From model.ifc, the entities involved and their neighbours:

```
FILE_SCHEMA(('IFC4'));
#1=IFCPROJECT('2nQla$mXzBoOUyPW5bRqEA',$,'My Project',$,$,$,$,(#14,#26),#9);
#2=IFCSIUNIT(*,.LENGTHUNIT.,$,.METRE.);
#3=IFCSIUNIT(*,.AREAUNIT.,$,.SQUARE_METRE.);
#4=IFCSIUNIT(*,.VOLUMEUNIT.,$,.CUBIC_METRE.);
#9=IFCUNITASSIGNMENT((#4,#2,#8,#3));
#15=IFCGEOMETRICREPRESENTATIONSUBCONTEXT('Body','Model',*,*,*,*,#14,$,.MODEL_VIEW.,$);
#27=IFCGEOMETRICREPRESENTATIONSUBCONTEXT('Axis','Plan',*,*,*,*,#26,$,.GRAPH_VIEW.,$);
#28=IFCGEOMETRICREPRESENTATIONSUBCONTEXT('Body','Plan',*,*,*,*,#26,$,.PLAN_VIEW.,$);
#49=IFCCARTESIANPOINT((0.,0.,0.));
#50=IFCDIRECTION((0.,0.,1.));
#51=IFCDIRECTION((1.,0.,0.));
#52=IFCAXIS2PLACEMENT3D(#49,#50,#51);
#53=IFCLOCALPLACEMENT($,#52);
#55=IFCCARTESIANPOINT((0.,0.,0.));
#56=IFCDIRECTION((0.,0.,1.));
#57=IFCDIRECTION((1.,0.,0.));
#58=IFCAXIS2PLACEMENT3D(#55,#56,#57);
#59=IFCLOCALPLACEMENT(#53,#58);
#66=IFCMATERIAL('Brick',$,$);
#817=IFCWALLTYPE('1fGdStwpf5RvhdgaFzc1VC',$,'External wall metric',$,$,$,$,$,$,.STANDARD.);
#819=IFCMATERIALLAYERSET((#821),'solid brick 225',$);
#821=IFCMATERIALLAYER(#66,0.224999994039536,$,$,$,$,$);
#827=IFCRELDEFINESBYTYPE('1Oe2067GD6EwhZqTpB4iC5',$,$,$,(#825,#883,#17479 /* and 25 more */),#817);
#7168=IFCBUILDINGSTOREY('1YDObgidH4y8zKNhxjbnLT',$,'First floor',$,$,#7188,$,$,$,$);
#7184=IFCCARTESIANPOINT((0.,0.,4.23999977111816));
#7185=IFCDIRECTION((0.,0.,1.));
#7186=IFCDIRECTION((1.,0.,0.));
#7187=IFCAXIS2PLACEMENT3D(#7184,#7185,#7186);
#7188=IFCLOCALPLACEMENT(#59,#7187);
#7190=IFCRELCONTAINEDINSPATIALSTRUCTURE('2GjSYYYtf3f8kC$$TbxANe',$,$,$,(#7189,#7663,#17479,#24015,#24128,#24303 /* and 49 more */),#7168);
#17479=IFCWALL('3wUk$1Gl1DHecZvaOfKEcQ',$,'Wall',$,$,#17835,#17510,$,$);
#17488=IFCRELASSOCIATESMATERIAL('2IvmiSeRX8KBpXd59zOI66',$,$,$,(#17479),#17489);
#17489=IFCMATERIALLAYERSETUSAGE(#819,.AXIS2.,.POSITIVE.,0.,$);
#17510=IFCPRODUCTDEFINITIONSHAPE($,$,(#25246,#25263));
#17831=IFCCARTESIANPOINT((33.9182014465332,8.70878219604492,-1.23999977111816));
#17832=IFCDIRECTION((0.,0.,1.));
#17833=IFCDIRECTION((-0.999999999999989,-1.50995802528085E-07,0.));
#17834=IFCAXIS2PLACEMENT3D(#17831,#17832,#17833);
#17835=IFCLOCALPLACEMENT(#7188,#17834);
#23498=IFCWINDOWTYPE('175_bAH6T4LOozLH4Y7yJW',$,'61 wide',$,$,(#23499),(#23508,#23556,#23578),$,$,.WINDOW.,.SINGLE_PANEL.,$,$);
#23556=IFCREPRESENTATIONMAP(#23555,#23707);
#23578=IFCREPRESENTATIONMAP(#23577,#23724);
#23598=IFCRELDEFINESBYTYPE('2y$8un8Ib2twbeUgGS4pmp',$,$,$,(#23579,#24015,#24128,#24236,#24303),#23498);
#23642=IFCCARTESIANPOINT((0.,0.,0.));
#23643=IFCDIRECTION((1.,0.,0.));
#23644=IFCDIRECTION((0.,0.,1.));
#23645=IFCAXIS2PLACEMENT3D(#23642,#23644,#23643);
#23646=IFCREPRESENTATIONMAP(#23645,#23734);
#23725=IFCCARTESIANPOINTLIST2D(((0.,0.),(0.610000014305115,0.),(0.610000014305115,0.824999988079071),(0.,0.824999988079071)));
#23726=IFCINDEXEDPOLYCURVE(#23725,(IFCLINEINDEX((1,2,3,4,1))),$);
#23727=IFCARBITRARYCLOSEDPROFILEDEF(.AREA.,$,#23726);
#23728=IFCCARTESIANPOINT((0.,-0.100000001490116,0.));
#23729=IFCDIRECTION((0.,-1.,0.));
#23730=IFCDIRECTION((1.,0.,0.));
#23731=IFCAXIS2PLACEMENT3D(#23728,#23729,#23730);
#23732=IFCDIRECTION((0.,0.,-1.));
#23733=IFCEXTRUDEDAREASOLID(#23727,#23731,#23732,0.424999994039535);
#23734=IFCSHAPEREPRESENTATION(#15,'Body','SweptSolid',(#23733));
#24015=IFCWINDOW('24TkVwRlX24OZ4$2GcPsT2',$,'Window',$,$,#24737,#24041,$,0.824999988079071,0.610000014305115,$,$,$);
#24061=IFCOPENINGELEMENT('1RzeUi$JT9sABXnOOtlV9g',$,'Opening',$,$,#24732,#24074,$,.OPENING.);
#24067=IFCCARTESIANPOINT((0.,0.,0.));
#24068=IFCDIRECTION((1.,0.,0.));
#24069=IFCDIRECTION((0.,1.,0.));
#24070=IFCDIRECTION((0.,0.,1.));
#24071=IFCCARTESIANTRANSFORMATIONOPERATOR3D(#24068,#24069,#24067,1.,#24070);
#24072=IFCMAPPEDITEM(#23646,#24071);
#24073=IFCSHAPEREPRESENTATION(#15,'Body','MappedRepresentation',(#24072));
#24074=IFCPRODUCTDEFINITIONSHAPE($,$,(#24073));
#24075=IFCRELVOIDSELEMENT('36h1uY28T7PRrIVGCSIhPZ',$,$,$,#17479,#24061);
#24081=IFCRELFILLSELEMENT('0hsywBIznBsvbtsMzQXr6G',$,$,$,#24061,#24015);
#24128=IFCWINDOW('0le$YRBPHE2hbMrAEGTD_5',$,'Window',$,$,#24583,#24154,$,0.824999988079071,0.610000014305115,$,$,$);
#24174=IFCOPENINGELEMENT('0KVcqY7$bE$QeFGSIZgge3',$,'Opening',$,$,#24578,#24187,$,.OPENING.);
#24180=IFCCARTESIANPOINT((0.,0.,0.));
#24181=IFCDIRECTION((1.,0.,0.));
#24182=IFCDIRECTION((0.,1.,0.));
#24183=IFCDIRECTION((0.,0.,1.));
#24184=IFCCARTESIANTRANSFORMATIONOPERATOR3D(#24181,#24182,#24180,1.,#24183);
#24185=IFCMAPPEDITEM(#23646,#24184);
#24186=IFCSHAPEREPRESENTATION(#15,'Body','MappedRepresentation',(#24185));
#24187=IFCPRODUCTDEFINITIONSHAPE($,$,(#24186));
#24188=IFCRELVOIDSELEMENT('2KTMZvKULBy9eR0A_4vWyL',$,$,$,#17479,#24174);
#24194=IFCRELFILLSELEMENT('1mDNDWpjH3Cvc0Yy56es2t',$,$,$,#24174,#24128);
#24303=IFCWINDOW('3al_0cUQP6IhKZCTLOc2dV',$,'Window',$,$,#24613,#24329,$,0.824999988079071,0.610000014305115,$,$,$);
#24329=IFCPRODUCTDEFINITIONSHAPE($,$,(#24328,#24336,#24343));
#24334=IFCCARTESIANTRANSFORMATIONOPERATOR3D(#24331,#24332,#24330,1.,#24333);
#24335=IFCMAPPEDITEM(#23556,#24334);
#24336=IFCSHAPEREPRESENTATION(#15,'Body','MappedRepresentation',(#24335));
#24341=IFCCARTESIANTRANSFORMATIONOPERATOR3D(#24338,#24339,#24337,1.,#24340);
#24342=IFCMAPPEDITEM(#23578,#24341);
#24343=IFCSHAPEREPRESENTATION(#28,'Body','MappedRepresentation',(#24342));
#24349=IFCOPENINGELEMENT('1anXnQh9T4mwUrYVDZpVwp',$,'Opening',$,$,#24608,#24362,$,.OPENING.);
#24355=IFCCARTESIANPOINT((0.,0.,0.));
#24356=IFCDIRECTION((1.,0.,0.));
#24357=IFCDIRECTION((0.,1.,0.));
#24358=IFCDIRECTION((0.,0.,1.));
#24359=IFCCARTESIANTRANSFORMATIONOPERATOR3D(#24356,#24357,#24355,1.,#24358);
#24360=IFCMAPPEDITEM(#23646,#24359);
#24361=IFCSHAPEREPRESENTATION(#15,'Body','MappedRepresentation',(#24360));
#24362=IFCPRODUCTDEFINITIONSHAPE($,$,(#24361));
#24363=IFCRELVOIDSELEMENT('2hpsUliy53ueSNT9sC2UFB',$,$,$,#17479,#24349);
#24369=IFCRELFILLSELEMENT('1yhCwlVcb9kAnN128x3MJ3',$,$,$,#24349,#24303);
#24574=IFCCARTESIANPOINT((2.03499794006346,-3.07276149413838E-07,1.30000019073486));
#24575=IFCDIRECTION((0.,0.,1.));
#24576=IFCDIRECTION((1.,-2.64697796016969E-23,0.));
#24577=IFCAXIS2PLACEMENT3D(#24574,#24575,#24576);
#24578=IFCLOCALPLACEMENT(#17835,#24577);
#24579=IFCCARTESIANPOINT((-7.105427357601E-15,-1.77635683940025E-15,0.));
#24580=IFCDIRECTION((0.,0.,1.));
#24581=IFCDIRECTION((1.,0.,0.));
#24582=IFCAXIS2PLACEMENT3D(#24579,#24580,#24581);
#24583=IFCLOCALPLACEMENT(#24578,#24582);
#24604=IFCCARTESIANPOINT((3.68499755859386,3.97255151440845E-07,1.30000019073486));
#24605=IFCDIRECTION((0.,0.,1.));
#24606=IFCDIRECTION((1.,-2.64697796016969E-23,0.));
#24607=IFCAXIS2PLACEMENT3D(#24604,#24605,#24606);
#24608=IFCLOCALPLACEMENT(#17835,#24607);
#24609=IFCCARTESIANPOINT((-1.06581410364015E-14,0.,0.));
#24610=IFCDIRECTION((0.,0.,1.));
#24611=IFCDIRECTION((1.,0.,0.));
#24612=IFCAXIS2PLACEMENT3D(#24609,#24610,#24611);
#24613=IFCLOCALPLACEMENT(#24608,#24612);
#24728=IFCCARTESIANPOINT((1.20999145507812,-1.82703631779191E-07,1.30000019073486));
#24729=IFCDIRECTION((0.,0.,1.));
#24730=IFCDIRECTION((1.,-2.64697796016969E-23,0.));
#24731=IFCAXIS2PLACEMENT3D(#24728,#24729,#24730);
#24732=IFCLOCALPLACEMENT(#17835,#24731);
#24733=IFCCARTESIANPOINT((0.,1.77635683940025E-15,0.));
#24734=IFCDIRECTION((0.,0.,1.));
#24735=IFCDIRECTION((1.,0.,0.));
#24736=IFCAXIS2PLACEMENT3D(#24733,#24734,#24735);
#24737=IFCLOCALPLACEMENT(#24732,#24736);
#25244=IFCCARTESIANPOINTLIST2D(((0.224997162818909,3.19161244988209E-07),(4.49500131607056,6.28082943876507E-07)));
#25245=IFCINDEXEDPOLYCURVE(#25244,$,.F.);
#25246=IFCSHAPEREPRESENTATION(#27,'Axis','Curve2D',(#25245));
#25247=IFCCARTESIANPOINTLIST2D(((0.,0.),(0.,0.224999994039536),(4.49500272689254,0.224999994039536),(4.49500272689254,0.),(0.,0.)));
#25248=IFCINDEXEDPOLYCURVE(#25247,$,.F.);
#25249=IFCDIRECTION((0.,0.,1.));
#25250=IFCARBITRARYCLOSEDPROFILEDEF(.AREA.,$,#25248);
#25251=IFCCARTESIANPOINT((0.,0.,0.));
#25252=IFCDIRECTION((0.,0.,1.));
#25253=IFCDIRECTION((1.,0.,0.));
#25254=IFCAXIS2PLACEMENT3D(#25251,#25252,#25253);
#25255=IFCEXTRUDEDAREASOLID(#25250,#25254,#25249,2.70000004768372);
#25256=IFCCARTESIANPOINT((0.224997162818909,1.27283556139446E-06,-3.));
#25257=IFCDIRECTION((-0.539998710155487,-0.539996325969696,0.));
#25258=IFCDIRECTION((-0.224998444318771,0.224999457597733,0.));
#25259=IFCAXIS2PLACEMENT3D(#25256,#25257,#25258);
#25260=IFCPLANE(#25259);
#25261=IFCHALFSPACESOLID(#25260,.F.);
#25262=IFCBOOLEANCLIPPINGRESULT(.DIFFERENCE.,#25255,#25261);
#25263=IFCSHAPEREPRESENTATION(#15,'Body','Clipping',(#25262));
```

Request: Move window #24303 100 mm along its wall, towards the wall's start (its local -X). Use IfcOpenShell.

```python
import ifcopenshell
import ifcopenshell.api.geometry
import ifcopenshell.util.placement
import ifcopenshell.util.unit

model = ifcopenshell.open("model.ifc")
unit_scale = ifcopenshell.util.unit.calculate_unit_scale(model)

window = model.by_guid("3al_0cUQP6IhKZCTLOc2dV")
opening = window.FillsVoids[0].RelatingOpeningElement
wall = opening.VoidsElements[0].RelatingBuildingElement

wall_matrix = ifcopenshell.util.placement.get_local_placement(wall.ObjectPlacement)
shift = wall_matrix[:3, 0] * -0.1 / unit_scale
before = ifcopenshell.util.placement.get_local_placement(window.ObjectPlacement)[:3, 3].copy()

# The window is placed relative to its opening, so it follows when the opening moves.
matrix = ifcopenshell.util.placement.get_local_placement(opening.ObjectPlacement)
matrix[:3, 3] += shift
ifcopenshell.api.geometry.edit_object_placement(
    model, product=opening, matrix=matrix, is_si=False, should_transform_children=True
)

after = ifcopenshell.util.placement.get_local_placement(window.ObjectPlacement)[:3, 3]
print("window moved by", (after - before).round(3) + 0.0)

model.write("model_rev.ifc")
```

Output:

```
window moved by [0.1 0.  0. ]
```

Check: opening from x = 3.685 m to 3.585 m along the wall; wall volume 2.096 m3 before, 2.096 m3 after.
